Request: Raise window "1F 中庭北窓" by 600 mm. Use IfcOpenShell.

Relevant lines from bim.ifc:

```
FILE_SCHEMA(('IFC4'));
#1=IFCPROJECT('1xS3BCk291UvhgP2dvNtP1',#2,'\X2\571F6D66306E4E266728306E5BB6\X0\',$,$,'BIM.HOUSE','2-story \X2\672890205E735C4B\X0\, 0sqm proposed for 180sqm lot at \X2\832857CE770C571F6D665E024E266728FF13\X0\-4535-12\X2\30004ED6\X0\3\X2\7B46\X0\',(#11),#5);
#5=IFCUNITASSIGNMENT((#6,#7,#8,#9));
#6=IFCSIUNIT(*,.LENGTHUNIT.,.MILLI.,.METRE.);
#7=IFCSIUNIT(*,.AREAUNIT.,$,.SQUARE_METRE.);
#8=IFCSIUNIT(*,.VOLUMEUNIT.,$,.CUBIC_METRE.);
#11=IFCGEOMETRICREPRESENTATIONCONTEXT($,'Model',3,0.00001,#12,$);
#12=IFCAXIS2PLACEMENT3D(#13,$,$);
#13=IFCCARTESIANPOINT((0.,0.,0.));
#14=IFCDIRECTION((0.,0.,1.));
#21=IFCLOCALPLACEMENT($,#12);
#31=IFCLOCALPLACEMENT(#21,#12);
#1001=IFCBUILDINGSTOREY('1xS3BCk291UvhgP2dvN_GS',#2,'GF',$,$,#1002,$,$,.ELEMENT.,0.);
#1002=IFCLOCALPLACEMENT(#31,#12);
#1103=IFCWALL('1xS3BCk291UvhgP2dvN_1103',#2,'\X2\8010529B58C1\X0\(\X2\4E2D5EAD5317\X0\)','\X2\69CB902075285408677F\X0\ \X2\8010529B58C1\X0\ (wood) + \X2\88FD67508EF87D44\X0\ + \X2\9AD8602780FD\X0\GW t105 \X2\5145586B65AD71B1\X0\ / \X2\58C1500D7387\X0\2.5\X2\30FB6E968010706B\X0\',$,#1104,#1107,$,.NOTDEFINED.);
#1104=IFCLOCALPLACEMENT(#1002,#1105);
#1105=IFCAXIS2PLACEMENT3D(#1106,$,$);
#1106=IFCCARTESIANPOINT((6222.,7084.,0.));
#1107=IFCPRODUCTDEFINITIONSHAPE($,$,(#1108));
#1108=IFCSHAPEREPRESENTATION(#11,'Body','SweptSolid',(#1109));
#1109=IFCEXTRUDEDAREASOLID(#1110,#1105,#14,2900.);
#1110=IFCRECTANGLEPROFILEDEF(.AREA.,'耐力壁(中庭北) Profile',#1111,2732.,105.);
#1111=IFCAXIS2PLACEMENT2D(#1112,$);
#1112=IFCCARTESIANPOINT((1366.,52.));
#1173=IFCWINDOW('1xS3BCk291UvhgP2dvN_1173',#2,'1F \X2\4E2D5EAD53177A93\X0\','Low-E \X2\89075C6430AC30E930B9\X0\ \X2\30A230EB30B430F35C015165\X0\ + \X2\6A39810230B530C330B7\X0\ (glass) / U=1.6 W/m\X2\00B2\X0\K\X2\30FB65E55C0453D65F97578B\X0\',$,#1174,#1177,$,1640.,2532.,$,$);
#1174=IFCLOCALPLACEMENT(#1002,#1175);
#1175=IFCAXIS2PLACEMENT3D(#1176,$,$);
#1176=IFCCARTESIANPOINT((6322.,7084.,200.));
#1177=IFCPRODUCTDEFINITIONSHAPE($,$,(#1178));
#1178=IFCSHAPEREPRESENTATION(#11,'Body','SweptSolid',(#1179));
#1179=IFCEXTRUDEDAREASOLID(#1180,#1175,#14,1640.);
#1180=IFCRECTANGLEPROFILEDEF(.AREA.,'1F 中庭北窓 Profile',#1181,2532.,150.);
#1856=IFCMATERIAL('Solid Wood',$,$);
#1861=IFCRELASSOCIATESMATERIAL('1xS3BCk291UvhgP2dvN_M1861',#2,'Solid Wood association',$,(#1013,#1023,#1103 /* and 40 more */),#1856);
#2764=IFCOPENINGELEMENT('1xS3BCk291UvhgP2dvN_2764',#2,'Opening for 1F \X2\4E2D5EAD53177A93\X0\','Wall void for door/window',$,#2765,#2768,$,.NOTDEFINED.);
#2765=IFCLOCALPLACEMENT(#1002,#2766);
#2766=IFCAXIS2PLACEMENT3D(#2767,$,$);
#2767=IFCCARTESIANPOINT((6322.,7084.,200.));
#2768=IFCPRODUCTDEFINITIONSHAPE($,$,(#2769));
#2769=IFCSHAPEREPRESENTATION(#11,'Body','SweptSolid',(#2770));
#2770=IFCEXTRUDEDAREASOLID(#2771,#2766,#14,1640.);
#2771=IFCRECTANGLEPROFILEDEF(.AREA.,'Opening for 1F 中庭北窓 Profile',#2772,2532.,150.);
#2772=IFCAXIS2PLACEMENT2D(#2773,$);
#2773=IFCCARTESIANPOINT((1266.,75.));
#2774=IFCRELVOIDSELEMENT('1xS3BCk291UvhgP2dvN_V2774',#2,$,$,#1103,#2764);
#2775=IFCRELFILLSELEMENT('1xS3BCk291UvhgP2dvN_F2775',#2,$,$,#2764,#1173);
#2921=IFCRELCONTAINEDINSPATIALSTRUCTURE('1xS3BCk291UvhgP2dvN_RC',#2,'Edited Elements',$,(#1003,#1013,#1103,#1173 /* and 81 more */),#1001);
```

```python
import numpy as np
import ifcopenshell
import ifcopenshell.api.geometry
import ifcopenshell.util.placement
import ifcopenshell.util.unit

model = ifcopenshell.open("bim.ifc")
unit_scale = ifcopenshell.util.unit.calculate_unit_scale(model)

window = model.by_guid("1xS3BCk291UvhgP2dvN_1173")
opening = window.FillsVoids[0].RelatingOpeningElement
dz = 0.6 / unit_scale

shift = np.array([0.0, 0.0, dz])
# The window is not placed relative to its opening, so move both.
for product in (opening, window):
    matrix = ifcopenshell.util.placement.get_local_placement(product.ObjectPlacement)
    matrix[:3, 3] += shift
    ifcopenshell.api.geometry.edit_object_placement(model, product=product, matrix=matrix, is_si=False)

print(f"moved by {dz * unit_scale:+.3f} m")

model.write("bim_edited.ifc")
```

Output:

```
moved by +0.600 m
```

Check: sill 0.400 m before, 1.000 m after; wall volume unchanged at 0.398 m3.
